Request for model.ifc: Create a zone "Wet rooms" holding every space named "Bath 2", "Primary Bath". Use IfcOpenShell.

First a look at what the model holds.

```python
import ifcopenshell

model = ifcopenshell.open("model.ifc")
print(model.schema)
seen = {}
for space in model.by_type("IfcSpace"):
    seen[space.LongName] = seen.get(space.LongName, 0) + 1
for name, count in sorted(seen.items(), key=str):
    print(count, "x", name)
print("zones:", [z.Name for z in model.by_type("IfcZone")][:20])
```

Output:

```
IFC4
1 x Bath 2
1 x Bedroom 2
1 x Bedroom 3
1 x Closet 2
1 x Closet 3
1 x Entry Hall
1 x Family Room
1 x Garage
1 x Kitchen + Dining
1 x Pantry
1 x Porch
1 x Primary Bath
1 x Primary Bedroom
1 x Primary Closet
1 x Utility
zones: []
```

```python
import ifcopenshell
import ifcopenshell.api.group
import ifcopenshell.api.root

model = ifcopenshell.open("model.ifc")

names = {"Bath 2", "Primary Bath"}
spaces = [s for s in model.by_type("IfcSpace") if s.LongName in names]

zone = ifcopenshell.api.root.create_entity(model, ifc_class="IfcZone", name="Wet rooms")
ifcopenshell.api.group.assign_group(model, products=spaces, group=zone)
print(len(spaces), "spaces in", zone.Name)

model.write("model_edited.ifc")
```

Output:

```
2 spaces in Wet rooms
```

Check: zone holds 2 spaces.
